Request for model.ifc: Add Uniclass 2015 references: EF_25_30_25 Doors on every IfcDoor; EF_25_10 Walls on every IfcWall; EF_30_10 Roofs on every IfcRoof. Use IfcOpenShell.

First a look at what the model holds.

```python
import ifcopenshell

model = ifcopenshell.open("model.ifc")
print(model.schema)
print("classifications:", [c.Name for c in model.by_type("IfcClassification")])
for ifc_class in ("IfcDoor", "IfcRoof", "IfcStair", "IfcWall", "IfcWindow"):
    print(ifc_class, len(model.by_type(ifc_class)))
```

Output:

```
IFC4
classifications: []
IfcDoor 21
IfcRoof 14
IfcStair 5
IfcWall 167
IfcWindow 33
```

```python
import ifcopenshell
import ifcopenshell.api.classification

model = ifcopenshell.open("model.ifc")

system = ifcopenshell.api.classification.add_classification(model, classification="Uniclass 2015")

codes = {
    "IfcDoor": ("EF_25_30_25", "Doors"),
    "IfcWall": ("EF_25_10", "Walls"),
    "IfcRoof": ("EF_30_10", "Roofs"),
}
for ifc_class, (code, name) in codes.items():
    products = model.by_type(ifc_class)
    ifcopenshell.api.classification.add_reference(
        model, products=products, classification=system, identification=code, name=name
    )
    print(code, len(products))

model.write("model_updated.ifc")
```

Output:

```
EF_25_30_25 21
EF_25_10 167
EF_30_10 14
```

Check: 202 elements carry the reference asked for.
